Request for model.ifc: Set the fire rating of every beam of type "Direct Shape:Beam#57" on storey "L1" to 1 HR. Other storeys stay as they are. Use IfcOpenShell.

First a look at what the model holds.

```python
import ifcopenshell
import ifcopenshell.util.element

model = ifcopenshell.open("model.ifc")
print(model.schema)
storey = next(s for s in model.by_type("IfcBuildingStorey") if s.Name == "L1")
beams = [e for e in ifcopenshell.util.element.get_decomposition(storey) if e.is_a("IfcBeam")]
seen = {}
for e in beams:
    element_type = ifcopenshell.util.element.get_type(e)
    key = (element_type.Name if element_type != e and element_type else None, ifcopenshell.util.element.get_pset(e, "Pset_BeamCommon", "FireRating"))
    seen[key] = seen.get(key, 0) + 1
for (name, value), count in sorted(seen.items(), key=str):
    print(count, "x", name, "|", value)
```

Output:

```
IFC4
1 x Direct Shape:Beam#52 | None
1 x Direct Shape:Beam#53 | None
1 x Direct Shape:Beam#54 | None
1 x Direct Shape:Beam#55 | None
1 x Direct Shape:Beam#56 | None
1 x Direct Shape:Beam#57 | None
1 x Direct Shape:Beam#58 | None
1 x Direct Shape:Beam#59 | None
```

```python
import ifcopenshell
import ifcopenshell.api.pset
import ifcopenshell.util.element

model = ifcopenshell.open("model.ifc")

storey = next(s for s in model.by_type("IfcBuildingStorey") if s.Name == "L1")
beams = [e for e in ifcopenshell.util.element.get_decomposition(storey) if e.is_a("IfcBeam")]

count = 0
for e in beams:
    element_type = ifcopenshell.util.element.get_type(e)
    if element_type in (None, e) or element_type.Name != "Direct Shape:Beam#57":
        continue
    # add_pset returns the element's existing set when there is one.
    pset = ifcopenshell.api.pset.add_pset(model, product=e, name="Pset_BeamCommon")
    ifcopenshell.api.pset.edit_pset(model, pset=pset, properties={"FireRating": "1 HR"})
    count += 1

print(count, "beams updated")

model.write("model_edited.ifc")
```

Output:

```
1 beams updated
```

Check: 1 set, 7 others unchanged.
